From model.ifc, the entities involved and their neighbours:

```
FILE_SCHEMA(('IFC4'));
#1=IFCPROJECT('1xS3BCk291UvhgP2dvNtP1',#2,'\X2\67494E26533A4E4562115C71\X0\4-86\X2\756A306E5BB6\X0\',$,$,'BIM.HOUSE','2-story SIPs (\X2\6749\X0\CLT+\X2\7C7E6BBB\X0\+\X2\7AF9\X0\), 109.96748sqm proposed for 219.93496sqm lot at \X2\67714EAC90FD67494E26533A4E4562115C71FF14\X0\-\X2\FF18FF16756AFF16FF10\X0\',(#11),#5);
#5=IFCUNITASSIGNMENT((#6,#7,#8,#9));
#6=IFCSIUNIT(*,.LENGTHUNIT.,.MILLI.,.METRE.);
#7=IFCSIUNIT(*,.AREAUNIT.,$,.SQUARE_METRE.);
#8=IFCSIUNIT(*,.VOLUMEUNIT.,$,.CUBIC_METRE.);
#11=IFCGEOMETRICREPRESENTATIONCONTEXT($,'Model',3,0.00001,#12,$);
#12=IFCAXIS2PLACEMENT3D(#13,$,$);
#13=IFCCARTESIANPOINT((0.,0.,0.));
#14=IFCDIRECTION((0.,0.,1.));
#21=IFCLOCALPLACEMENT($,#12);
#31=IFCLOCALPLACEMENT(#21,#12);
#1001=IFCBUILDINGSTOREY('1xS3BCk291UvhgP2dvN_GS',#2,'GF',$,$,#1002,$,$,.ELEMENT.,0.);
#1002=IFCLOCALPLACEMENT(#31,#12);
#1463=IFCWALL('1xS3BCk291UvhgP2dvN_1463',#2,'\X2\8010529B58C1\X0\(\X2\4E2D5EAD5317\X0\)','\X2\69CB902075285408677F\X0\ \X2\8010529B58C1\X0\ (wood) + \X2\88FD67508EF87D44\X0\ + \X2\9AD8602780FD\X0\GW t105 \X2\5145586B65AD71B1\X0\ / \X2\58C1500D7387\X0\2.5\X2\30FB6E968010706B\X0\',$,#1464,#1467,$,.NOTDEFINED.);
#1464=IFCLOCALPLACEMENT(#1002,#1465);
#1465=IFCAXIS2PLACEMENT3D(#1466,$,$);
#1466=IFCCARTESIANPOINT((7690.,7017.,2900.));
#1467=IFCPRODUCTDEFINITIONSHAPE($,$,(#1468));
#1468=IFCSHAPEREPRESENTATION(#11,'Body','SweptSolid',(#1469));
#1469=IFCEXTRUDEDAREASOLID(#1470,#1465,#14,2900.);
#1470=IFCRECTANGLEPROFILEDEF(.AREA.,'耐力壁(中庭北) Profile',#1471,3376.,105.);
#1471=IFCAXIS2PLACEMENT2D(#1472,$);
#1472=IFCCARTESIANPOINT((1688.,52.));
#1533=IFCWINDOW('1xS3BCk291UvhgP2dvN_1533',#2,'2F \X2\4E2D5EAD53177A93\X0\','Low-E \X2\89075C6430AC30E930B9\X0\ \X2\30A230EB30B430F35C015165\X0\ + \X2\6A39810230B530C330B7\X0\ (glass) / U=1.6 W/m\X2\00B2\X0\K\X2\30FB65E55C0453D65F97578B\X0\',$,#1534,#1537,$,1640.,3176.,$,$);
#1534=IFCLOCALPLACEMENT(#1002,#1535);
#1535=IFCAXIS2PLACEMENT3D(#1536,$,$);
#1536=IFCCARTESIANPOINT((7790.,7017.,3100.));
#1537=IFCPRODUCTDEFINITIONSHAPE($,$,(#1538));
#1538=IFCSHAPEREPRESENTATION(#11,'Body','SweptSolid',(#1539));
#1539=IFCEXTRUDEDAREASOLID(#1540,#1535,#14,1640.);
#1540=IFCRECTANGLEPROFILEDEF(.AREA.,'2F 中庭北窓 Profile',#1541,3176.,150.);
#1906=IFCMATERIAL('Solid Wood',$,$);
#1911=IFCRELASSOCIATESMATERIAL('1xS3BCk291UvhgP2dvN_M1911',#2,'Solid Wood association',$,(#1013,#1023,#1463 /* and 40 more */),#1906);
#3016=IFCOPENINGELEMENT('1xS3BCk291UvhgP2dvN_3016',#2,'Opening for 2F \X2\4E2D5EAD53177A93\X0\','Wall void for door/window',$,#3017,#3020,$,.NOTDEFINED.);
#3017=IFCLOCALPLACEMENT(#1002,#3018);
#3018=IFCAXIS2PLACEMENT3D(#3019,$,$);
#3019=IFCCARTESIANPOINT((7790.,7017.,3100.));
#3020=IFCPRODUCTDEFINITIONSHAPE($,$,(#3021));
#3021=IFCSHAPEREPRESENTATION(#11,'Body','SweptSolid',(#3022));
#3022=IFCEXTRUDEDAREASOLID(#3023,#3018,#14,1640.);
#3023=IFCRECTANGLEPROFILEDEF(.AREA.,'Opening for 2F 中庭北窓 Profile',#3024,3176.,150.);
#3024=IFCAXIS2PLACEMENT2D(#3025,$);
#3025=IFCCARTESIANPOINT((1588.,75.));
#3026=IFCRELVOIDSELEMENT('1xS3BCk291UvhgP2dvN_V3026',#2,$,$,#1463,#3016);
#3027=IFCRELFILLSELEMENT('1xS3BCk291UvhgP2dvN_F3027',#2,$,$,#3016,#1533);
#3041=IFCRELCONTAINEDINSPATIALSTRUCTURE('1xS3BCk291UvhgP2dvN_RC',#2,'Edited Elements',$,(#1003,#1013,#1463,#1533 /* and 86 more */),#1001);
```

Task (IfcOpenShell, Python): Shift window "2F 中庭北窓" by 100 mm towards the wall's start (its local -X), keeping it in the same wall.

```python
import ifcopenshell
import ifcopenshell.api.geometry
import ifcopenshell.util.placement
import ifcopenshell.util.unit

model = ifcopenshell.open("model.ifc")
unit_scale = ifcopenshell.util.unit.calculate_unit_scale(model)

window = model.by_guid("1xS3BCk291UvhgP2dvN_1533")
opening = window.FillsVoids[0].RelatingOpeningElement
wall = opening.VoidsElements[0].RelatingBuildingElement

wall_matrix = ifcopenshell.util.placement.get_local_placement(wall.ObjectPlacement)
shift = wall_matrix[:3, 0] * -0.1 / unit_scale
before = ifcopenshell.util.placement.get_local_placement(window.ObjectPlacement)[:3, 3].copy()

# The window is not placed relative to its opening, so move both.
for product in (opening, window):
    matrix = ifcopenshell.util.placement.get_local_placement(product.ObjectPlacement)
    matrix[:3, 3] += shift
    ifcopenshell.api.geometry.edit_object_placement(model, product=product, matrix=matrix, is_si=False)

after = ifcopenshell.util.placement.get_local_placement(window.ObjectPlacement)[:3, 3]
print("window moved by", (after - before).round(3) + 0.0)

model.write("model_updated.ifc")
```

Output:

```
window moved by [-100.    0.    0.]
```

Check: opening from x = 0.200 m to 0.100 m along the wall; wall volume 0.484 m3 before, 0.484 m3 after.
